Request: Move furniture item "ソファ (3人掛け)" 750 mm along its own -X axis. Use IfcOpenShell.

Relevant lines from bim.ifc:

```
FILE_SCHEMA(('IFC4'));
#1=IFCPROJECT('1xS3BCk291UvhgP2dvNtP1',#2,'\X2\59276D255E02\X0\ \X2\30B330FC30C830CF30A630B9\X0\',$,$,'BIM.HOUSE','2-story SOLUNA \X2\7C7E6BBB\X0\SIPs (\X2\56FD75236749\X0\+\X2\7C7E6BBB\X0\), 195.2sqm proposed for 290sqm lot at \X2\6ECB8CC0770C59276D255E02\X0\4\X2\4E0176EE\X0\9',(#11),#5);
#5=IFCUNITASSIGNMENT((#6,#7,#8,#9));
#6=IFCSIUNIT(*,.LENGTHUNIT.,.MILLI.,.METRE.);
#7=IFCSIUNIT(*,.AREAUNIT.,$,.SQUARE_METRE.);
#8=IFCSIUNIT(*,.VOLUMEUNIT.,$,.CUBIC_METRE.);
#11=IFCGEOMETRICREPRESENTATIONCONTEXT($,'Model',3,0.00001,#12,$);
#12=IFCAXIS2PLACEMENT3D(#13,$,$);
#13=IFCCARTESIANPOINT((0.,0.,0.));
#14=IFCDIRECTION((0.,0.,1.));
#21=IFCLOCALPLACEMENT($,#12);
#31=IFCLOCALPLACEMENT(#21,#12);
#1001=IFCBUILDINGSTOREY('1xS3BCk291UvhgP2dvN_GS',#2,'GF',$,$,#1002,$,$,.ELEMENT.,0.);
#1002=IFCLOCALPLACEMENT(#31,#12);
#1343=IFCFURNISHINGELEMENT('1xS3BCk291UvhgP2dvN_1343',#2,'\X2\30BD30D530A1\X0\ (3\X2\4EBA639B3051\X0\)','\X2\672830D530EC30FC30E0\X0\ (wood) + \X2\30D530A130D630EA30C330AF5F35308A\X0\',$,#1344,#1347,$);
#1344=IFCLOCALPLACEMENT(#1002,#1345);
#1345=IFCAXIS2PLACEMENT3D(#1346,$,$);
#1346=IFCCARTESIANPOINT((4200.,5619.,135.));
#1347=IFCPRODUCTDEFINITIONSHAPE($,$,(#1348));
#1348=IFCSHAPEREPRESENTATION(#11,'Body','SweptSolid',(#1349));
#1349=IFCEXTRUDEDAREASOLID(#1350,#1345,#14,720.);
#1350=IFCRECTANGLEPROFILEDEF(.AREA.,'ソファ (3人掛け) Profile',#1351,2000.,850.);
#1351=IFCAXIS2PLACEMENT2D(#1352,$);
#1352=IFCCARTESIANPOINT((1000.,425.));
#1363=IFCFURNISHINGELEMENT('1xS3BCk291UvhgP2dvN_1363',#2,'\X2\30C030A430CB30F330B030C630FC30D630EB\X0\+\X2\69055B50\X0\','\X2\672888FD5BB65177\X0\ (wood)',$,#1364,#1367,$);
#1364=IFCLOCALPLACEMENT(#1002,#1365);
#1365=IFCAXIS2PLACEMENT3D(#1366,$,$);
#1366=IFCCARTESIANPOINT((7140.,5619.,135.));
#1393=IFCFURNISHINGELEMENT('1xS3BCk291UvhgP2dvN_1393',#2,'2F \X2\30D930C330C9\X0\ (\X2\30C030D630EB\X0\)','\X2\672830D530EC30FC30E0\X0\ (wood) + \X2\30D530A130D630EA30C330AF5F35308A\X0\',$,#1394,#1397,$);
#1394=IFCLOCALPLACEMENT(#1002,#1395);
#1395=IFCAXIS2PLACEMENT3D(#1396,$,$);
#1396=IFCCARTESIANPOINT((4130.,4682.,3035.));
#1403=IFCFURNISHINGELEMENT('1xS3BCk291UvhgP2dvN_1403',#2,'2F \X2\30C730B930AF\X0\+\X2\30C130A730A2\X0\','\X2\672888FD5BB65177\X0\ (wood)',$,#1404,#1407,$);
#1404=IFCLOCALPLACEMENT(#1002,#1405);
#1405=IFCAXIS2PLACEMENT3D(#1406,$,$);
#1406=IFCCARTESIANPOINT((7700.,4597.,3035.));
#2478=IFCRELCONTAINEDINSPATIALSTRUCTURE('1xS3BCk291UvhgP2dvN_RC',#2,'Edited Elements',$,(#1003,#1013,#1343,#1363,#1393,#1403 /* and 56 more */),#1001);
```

```python
import ifcopenshell
import ifcopenshell.api.geometry
import ifcopenshell.util.placement
import ifcopenshell.util.unit

model = ifcopenshell.open("bim.ifc")
unit_scale = ifcopenshell.util.unit.calculate_unit_scale(model)

item = model.by_guid("1xS3BCk291UvhgP2dvN_1343")
matrix = ifcopenshell.util.placement.get_local_placement(item.ObjectPlacement)
matrix[:3, 3] -= matrix[:3, 0] * 0.75 / unit_scale
ifcopenshell.api.geometry.edit_object_placement(model, product=item, matrix=matrix, is_si=False)

print(ifcopenshell.util.placement.get_local_placement(item.ObjectPlacement).round(3) + 0.0)

model.write("bim-out.ifc")
```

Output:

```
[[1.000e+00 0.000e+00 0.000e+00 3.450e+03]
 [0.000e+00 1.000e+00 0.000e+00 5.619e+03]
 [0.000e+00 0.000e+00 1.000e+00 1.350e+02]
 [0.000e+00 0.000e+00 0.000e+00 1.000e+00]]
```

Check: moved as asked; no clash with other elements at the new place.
